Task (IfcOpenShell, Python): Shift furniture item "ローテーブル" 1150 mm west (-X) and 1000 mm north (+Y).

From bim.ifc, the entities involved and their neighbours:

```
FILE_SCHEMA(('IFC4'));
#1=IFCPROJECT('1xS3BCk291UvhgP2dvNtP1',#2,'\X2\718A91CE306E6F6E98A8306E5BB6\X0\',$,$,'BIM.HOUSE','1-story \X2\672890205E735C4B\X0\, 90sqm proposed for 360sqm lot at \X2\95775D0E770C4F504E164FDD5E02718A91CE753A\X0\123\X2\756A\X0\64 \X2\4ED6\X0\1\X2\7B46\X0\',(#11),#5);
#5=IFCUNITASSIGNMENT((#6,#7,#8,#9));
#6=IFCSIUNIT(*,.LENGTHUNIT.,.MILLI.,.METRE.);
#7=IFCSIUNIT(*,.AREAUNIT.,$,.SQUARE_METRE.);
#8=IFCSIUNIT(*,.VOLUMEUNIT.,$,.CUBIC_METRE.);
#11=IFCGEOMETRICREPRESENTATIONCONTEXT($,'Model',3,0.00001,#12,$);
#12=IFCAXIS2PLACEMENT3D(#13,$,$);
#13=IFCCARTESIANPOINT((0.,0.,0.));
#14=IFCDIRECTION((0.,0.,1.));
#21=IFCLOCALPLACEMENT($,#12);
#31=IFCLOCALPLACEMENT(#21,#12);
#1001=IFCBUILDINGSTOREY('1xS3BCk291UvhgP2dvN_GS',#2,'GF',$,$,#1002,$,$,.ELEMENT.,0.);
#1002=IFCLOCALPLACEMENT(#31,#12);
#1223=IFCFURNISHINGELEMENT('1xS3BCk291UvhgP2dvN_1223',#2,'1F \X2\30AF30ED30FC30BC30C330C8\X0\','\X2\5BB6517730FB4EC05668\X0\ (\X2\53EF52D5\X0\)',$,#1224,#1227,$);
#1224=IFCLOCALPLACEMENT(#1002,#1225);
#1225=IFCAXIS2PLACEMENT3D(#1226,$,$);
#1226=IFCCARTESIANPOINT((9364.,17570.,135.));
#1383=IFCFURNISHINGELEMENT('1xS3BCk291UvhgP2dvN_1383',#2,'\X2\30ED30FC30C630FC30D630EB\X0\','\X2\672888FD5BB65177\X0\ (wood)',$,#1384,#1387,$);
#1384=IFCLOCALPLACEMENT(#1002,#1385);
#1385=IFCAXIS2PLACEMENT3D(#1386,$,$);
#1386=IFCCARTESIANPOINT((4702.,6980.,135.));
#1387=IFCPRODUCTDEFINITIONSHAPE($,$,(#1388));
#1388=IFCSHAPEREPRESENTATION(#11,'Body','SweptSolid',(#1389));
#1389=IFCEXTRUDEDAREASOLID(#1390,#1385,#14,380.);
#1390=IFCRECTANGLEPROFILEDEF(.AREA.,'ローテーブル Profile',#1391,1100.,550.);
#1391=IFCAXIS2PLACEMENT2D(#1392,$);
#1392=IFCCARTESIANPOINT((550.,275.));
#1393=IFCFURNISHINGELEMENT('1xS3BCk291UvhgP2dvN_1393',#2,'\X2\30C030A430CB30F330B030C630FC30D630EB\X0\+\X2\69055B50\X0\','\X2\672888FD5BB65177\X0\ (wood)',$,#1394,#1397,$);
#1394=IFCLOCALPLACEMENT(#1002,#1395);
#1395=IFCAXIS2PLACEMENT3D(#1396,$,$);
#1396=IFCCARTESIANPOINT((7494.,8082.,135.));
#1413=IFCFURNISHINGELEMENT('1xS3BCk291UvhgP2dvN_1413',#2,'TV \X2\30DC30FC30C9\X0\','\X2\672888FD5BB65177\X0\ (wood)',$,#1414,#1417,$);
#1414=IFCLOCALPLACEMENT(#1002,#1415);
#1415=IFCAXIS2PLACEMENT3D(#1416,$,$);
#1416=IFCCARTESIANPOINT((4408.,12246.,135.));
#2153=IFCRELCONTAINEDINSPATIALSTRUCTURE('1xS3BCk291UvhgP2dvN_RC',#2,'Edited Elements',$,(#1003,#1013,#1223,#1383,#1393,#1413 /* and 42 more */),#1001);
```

```python
import ifcopenshell
import ifcopenshell.api.geometry
import ifcopenshell.util.placement

model = ifcopenshell.open("bim.ifc")

item = model.by_guid("1xS3BCk291UvhgP2dvN_1383")
matrix = ifcopenshell.util.placement.get_local_placement(item.ObjectPlacement)
matrix[0, 3] -= 1150.0
matrix[1, 3] += 1000.0
ifcopenshell.api.geometry.edit_object_placement(model, product=item, matrix=matrix, is_si=False)

print(ifcopenshell.util.placement.get_local_placement(item.ObjectPlacement).round(3) + 0.0)

model.write("bim-out.ifc")
```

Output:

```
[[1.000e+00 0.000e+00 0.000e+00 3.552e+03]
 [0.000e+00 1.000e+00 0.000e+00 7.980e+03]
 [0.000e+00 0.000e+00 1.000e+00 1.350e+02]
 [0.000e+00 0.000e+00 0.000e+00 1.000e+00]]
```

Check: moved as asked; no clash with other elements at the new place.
